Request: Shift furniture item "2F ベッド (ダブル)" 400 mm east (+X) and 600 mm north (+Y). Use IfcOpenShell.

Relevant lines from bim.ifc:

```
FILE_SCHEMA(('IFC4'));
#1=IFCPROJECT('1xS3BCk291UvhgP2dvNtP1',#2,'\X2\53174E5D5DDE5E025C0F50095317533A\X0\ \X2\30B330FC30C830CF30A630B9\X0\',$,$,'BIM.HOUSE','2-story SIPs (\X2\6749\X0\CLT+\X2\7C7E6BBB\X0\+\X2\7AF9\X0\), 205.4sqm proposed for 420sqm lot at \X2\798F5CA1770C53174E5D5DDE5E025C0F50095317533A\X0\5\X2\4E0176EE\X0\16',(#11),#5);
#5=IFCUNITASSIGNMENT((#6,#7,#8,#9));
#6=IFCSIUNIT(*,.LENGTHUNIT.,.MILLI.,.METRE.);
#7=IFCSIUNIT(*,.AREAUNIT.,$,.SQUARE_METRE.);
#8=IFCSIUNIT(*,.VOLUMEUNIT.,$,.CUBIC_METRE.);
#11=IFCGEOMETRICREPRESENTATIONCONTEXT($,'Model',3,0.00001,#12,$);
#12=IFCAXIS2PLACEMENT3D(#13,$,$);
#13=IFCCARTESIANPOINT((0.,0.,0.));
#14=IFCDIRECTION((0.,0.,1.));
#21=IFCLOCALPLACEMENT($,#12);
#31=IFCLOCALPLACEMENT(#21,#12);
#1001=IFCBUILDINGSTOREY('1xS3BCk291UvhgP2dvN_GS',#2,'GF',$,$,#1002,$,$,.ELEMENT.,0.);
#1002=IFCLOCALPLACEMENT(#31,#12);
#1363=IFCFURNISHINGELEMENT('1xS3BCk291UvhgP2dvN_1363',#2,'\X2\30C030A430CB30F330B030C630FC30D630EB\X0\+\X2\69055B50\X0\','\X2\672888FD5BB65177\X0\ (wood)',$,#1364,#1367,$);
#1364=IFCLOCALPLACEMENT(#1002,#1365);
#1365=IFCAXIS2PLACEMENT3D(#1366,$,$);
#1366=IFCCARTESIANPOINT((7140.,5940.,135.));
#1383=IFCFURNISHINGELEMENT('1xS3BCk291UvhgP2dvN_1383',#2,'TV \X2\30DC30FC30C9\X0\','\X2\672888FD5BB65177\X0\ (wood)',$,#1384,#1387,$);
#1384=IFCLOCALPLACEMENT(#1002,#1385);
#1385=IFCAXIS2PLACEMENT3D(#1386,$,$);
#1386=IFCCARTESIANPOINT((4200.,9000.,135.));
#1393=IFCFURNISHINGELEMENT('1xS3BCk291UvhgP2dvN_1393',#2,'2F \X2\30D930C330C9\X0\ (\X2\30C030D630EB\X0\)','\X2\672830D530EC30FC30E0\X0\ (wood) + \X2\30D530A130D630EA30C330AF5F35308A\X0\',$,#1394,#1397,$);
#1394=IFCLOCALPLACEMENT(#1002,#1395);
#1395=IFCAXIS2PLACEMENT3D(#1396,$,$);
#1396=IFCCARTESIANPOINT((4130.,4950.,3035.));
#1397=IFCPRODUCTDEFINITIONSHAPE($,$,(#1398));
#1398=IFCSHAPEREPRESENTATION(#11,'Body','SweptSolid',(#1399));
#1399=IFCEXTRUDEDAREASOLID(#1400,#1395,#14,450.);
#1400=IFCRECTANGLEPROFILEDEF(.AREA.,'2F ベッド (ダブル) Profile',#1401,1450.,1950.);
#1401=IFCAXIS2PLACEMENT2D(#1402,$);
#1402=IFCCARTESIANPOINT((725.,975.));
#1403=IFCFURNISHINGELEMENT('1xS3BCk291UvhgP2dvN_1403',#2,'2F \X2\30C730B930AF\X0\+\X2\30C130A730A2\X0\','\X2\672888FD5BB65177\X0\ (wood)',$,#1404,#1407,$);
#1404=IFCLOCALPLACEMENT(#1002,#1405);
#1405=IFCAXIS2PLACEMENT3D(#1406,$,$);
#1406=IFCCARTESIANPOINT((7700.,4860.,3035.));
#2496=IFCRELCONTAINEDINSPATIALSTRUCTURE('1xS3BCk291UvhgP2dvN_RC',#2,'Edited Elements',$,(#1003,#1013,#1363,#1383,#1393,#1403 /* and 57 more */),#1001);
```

```python
import ifcopenshell
import ifcopenshell.api.geometry
import ifcopenshell.util.placement

model = ifcopenshell.open("bim.ifc")

item = model.by_guid("1xS3BCk291UvhgP2dvN_1393")
matrix = ifcopenshell.util.placement.get_local_placement(item.ObjectPlacement)
matrix[0, 3] += 400.0
matrix[1, 3] += 600.0
ifcopenshell.api.geometry.edit_object_placement(model, product=item, matrix=matrix, is_si=False)

print(ifcopenshell.util.placement.get_local_placement(item.ObjectPlacement).round(3) + 0.0)

model.write("bim-out.ifc")
```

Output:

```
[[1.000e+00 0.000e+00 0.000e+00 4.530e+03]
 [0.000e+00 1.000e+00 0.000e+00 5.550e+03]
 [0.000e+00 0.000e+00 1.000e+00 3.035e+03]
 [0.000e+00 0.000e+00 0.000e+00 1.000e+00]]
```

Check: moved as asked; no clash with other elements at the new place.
